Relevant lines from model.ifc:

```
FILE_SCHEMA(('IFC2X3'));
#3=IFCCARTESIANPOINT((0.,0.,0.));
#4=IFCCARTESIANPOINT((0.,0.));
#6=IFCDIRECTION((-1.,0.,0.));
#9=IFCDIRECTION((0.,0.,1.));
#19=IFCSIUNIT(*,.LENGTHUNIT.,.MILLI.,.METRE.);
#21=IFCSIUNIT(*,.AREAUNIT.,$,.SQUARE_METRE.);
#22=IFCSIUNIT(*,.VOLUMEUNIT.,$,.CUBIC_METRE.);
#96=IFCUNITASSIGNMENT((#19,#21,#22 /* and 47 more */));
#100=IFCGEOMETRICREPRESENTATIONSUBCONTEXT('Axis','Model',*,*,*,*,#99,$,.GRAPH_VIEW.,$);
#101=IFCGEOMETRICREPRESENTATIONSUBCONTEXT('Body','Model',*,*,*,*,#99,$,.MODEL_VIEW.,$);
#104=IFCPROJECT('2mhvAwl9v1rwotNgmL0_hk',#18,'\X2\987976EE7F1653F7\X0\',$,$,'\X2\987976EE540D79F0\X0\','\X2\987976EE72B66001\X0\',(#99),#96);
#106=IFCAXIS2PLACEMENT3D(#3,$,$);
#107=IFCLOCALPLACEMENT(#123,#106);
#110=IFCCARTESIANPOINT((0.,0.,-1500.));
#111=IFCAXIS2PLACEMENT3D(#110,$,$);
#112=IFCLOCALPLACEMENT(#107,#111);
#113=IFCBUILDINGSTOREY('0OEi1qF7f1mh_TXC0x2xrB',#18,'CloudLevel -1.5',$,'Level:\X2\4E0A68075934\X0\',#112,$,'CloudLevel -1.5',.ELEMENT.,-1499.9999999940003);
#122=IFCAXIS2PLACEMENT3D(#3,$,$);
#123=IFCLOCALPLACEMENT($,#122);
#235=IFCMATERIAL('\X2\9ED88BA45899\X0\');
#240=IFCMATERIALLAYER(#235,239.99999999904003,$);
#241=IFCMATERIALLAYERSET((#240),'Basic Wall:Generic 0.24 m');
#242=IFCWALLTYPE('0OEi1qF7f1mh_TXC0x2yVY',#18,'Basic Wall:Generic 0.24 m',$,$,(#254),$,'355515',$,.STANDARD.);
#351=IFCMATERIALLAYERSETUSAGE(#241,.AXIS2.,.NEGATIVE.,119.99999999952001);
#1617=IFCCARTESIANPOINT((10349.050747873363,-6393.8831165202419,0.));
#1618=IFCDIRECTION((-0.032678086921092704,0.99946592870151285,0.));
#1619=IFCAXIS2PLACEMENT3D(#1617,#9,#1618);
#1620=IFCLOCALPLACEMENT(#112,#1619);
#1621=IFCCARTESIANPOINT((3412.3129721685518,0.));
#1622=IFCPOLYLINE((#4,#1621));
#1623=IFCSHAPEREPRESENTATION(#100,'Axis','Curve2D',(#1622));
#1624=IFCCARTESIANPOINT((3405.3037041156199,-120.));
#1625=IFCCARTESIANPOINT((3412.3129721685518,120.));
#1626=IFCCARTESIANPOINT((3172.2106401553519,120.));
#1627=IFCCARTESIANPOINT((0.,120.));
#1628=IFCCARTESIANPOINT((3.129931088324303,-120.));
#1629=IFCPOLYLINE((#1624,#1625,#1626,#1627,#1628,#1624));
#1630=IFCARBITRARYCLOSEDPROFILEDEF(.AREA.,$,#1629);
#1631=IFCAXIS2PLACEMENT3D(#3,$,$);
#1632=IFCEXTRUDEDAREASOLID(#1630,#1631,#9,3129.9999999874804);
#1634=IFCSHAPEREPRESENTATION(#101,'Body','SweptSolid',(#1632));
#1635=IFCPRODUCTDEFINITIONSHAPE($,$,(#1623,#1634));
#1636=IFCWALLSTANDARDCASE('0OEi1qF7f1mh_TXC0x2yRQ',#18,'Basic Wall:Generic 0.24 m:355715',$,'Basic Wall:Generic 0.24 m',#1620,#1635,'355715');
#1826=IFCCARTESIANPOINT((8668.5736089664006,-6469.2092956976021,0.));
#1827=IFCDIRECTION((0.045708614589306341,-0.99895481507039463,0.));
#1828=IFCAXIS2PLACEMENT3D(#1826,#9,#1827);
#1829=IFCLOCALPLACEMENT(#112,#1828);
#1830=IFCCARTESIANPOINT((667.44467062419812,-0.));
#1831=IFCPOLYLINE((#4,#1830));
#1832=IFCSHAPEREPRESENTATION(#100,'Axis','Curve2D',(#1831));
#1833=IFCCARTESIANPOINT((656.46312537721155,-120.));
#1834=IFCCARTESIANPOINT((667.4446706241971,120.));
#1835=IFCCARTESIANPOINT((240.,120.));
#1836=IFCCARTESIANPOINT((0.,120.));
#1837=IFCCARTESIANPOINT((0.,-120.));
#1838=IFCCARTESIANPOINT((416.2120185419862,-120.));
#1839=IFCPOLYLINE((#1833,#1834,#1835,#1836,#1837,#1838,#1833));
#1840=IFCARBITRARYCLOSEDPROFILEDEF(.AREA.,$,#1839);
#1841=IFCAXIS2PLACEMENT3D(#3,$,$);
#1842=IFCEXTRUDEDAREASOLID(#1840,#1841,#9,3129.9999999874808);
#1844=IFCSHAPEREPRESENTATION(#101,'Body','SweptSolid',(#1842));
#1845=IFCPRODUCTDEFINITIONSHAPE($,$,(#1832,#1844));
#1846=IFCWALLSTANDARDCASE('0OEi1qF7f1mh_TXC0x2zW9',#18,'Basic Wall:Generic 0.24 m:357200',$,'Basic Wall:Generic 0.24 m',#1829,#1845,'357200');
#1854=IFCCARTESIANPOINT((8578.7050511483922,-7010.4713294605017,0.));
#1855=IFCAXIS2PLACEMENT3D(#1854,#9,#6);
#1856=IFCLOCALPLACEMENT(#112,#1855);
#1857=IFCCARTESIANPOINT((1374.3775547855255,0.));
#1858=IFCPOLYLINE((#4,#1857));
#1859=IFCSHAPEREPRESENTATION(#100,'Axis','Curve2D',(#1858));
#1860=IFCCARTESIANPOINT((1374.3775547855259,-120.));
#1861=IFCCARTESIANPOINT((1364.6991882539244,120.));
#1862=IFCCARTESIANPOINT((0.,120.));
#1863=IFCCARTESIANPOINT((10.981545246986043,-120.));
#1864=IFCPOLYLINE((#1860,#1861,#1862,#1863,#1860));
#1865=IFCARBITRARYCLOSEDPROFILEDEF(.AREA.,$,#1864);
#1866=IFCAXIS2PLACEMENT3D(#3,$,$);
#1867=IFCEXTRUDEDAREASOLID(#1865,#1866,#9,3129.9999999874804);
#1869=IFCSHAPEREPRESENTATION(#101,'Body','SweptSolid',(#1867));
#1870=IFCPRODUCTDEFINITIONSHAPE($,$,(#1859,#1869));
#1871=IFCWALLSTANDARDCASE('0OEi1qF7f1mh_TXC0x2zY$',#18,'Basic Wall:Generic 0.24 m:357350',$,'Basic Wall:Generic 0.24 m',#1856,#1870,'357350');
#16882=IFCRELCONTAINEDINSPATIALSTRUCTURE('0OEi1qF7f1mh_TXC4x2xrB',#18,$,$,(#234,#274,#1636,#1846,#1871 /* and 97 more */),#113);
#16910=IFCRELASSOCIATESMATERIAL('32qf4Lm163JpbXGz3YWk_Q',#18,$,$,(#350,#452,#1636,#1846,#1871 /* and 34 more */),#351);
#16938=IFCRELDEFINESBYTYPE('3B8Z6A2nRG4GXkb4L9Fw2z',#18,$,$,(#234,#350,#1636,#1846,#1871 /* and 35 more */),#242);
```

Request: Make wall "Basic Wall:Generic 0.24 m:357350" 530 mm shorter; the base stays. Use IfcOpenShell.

```python
import ifcopenshell
import ifcopenshell.geom
import ifcopenshell.util.representation
import ifcopenshell.util.shape

model = ifcopenshell.open("model.ifc")
settings = ifcopenshell.geom.settings()


def volume(element):
    """Net volume in cubic metres, openings subtracted."""
    shape = ifcopenshell.geom.create_shape(settings, element)
    return ifcopenshell.util.shape.get_volume(shape.geometry)


wall = model.by_guid("0OEi1qF7f1mh_TXC0x2zY$")
before = volume(wall)

body = ifcopenshell.util.representation.get_representation(wall, "Model", "Body")
solid = body.Items[0]
old_height = solid.Depth
solid.Depth -= 530.0
after = volume(wall)

print(f"height {old_height:g} -> {solid.Depth:g}, volume {before:.3f} -> {after:.3f} m3")

model.write("model-out.ifc")
```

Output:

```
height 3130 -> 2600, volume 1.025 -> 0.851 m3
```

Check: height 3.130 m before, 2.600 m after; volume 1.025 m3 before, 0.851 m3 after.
